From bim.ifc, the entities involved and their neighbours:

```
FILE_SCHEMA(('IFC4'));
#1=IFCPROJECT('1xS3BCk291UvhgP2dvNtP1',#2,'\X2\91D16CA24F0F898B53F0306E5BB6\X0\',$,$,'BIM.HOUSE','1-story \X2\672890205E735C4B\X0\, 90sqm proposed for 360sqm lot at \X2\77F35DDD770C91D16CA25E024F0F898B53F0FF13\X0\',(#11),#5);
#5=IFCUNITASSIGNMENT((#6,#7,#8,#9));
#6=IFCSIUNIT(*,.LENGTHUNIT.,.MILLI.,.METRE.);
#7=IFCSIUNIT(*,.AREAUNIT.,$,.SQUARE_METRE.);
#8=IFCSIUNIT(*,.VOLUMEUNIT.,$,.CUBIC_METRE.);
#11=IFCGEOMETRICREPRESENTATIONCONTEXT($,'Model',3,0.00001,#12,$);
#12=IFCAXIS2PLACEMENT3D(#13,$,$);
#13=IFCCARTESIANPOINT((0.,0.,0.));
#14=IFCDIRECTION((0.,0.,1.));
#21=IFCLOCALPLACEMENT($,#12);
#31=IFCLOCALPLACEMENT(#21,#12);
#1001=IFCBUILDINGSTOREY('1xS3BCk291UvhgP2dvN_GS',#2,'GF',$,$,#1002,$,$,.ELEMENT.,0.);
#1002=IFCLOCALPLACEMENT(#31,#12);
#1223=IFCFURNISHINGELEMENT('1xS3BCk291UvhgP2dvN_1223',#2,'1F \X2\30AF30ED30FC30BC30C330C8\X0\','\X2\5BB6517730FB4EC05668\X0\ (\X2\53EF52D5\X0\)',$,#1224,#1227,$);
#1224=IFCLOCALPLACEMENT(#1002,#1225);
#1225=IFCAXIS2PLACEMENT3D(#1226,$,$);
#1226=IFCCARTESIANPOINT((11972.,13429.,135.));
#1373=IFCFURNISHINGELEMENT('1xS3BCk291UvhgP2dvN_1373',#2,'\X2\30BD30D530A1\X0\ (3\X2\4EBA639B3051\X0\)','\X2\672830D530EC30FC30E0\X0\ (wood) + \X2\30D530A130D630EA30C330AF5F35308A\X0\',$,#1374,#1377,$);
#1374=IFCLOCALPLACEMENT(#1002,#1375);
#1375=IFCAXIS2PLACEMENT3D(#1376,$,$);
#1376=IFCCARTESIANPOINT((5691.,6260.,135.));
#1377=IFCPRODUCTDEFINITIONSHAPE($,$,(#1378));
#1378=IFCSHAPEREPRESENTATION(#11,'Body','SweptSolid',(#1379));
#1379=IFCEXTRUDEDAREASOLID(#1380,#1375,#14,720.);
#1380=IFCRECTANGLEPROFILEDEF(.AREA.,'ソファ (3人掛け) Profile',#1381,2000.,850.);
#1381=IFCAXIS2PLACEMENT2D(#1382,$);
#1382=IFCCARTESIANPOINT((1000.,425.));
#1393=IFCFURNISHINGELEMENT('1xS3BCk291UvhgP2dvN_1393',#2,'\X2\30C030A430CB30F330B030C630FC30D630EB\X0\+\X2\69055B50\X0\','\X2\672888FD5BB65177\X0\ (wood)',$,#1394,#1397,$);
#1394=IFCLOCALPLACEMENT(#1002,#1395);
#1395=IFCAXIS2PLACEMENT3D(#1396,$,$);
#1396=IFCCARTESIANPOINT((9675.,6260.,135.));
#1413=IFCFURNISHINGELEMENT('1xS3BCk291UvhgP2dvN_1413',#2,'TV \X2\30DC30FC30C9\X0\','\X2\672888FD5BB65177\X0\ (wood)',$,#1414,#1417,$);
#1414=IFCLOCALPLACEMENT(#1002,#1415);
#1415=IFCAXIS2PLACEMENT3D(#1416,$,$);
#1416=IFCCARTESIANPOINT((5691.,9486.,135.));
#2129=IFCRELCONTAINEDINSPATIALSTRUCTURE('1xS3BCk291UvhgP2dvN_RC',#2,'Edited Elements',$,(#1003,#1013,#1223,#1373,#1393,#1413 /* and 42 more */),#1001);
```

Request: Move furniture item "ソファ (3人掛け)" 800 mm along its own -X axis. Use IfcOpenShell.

```python
import ifcopenshell
import ifcopenshell.api.geometry
import ifcopenshell.util.placement
import ifcopenshell.util.unit

model = ifcopenshell.open("bim.ifc")
unit_scale = ifcopenshell.util.unit.calculate_unit_scale(model)

item = model.by_guid("1xS3BCk291UvhgP2dvN_1373")
matrix = ifcopenshell.util.placement.get_local_placement(item.ObjectPlacement)
matrix[:3, 3] -= matrix[:3, 0] * 0.8 / unit_scale
ifcopenshell.api.geometry.edit_object_placement(model, product=item, matrix=matrix, is_si=False)

print(ifcopenshell.util.placement.get_local_placement(item.ObjectPlacement).round(3) + 0.0)

model.write("bim_updated.ifc")
```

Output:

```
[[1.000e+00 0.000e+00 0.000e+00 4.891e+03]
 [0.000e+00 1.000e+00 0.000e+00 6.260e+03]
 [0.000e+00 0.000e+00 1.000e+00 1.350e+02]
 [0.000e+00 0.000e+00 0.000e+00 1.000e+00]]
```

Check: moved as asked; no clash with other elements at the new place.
